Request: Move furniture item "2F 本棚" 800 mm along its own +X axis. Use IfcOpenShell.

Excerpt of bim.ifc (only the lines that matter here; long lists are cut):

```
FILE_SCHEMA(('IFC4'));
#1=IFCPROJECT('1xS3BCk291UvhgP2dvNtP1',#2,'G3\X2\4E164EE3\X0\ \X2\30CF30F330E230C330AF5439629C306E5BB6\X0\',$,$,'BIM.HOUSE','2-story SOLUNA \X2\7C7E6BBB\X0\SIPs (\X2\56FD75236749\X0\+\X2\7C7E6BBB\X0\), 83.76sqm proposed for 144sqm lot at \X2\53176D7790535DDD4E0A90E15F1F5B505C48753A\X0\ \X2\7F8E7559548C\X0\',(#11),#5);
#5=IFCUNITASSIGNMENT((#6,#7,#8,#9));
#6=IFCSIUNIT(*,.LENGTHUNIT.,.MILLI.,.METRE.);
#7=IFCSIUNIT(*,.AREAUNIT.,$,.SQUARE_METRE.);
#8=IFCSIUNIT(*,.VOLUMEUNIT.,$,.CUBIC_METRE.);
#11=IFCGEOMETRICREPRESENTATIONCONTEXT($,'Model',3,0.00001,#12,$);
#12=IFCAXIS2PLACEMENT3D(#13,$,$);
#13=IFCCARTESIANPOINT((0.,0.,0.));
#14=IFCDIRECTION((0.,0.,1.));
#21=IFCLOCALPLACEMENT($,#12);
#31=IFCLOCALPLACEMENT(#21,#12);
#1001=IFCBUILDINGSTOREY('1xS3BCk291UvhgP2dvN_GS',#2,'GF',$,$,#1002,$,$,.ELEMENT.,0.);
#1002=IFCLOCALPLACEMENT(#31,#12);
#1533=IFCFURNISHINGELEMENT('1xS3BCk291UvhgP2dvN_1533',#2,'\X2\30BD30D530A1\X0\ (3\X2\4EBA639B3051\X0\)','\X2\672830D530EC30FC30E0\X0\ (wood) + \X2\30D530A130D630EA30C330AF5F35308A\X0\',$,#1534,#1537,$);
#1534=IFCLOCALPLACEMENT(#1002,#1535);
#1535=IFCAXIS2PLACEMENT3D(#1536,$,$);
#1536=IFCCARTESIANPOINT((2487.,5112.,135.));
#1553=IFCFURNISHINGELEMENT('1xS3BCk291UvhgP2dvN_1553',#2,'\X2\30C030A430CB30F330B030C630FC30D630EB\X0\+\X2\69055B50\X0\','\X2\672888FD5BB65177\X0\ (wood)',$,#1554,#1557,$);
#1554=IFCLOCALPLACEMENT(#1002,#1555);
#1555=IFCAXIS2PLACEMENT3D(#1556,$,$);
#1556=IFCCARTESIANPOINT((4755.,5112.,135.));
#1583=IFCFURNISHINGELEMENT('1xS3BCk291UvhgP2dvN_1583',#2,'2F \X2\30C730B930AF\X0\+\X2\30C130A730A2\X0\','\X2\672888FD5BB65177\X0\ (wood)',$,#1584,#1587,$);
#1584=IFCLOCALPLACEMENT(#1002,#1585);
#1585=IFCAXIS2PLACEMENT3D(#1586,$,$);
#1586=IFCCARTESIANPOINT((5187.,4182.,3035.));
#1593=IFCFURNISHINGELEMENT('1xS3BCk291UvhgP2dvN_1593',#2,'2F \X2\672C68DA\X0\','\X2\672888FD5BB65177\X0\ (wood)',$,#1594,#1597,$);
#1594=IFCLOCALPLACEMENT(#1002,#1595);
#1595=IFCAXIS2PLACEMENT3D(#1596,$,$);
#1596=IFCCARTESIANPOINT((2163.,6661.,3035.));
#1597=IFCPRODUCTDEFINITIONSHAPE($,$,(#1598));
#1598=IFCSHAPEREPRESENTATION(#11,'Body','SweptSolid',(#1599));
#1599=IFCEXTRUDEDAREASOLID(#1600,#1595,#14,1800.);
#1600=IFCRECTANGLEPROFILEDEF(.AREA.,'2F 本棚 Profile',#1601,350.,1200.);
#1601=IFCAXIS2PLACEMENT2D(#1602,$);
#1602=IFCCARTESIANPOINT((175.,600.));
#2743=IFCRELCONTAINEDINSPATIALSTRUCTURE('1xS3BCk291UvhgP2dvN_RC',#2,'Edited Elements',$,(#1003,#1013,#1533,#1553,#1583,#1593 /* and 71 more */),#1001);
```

```python
import ifcopenshell
import ifcopenshell.api.geometry
import ifcopenshell.util.placement

model = ifcopenshell.open("bim.ifc")

item = model.by_id(1593)
matrix = ifcopenshell.util.placement.get_local_placement(item.ObjectPlacement)
matrix[:3, 3] += matrix[:3, 0] * 800.0
ifcopenshell.api.geometry.edit_object_placement(model, product=item, matrix=matrix, is_si=False)

print(ifcopenshell.util.placement.get_local_placement(item.ObjectPlacement).round(3) + 0.0)

model.write("bim_updated.ifc")
```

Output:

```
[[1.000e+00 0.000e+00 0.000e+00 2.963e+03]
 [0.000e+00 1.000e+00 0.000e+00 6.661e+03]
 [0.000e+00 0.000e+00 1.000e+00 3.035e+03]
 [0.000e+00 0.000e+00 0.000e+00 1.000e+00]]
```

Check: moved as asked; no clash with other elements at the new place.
